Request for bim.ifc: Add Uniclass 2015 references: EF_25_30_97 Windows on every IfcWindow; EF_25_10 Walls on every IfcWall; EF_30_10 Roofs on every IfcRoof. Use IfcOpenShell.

First a look at what the model holds.

```python
import ifcopenshell

model = ifcopenshell.open("bim.ifc")
print(model.schema)
print("classifications:", [c.Name for c in model.by_type("IfcClassification")])
for ifc_class in ("IfcDoor", "IfcRoof", "IfcStair", "IfcWall", "IfcWindow"):
    print(ifc_class, len(model.by_type(ifc_class)))
```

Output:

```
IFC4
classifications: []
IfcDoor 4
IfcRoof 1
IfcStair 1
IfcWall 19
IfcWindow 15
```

```python
import ifcopenshell
import ifcopenshell.api.classification

model = ifcopenshell.open("bim.ifc")

system = ifcopenshell.api.classification.add_classification(model, classification="Uniclass 2015")

codes = {
    "IfcWindow": ("EF_25_30_97", "Windows"),
    "IfcWall": ("EF_25_10", "Walls"),
    "IfcRoof": ("EF_30_10", "Roofs"),
}
for ifc_class, (code, name) in codes.items():
    products = model.by_type(ifc_class)
    ifcopenshell.api.classification.add_reference(
        model, products=products, classification=system, identification=code, name=name
    )
    print(code, len(products))

model.write("bim_updated.ifc")
```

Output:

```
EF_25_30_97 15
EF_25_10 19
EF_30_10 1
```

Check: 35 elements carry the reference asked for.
